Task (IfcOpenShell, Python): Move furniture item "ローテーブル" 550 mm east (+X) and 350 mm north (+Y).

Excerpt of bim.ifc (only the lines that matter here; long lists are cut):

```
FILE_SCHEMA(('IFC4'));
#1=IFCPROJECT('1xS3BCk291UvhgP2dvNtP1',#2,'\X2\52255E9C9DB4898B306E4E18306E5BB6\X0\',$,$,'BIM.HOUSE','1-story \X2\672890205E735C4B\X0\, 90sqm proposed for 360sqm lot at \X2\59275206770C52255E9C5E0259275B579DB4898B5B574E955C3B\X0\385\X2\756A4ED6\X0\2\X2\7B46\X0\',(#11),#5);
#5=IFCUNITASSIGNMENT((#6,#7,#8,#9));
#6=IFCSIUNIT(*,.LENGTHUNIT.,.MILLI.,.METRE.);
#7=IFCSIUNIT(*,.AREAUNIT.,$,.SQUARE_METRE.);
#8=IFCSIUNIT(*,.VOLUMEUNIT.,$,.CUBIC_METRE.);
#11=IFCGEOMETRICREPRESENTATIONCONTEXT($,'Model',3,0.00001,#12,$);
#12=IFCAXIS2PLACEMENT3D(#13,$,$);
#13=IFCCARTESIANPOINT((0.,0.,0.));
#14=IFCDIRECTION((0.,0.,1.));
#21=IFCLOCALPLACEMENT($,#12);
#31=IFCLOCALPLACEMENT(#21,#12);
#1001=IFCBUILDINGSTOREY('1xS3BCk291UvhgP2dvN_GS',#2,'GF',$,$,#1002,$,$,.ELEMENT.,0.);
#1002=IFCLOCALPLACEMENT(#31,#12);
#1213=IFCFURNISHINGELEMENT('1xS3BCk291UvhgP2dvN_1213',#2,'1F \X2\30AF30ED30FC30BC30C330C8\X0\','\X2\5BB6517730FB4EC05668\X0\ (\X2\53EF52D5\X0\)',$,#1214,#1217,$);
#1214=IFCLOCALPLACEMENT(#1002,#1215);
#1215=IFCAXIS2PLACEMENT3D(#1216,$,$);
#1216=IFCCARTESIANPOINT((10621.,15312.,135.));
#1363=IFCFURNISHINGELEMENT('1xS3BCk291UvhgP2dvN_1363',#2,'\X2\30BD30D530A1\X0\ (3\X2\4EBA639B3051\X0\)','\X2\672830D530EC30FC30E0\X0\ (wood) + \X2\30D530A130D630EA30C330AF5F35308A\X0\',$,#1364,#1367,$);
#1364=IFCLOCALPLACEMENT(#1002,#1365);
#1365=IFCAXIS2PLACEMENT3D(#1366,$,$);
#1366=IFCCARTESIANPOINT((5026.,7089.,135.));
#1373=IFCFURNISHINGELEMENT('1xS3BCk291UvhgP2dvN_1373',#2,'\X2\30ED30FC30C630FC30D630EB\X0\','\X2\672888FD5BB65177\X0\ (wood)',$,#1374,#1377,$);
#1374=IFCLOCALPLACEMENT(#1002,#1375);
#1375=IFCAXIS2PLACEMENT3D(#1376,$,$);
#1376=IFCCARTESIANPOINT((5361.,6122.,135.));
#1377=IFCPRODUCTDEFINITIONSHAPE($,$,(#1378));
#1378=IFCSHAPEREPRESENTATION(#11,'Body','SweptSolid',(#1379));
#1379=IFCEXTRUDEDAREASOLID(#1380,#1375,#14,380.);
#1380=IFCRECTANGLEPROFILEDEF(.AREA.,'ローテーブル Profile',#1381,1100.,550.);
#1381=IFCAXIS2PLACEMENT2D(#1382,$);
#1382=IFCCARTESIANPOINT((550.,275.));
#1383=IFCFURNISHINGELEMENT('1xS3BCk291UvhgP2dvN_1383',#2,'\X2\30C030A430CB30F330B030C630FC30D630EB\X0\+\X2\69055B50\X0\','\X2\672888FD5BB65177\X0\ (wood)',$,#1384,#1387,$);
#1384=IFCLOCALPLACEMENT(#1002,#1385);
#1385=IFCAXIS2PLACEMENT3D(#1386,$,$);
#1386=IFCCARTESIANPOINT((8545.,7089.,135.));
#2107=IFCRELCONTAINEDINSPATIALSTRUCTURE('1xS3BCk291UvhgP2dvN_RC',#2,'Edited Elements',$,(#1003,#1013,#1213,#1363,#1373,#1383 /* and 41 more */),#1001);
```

```python
import ifcopenshell
import ifcopenshell.api.geometry
import ifcopenshell.util.placement
import ifcopenshell.util.unit

model = ifcopenshell.open("bim.ifc")
unit_scale = ifcopenshell.util.unit.calculate_unit_scale(model)

item = model.by_guid("1xS3BCk291UvhgP2dvN_1373")
matrix = ifcopenshell.util.placement.get_local_placement(item.ObjectPlacement)
matrix[0, 3] += 0.55 / unit_scale
matrix[1, 3] += 0.35 / unit_scale
ifcopenshell.api.geometry.edit_object_placement(model, product=item, matrix=matrix, is_si=False)

print(ifcopenshell.util.placement.get_local_placement(item.ObjectPlacement).round(3) + 0.0)

model.write("bim-out.ifc")
```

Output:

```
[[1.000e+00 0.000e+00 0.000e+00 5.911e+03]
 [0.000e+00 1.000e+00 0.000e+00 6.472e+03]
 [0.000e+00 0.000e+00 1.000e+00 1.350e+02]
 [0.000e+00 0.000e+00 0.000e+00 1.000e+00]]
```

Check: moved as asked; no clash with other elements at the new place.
